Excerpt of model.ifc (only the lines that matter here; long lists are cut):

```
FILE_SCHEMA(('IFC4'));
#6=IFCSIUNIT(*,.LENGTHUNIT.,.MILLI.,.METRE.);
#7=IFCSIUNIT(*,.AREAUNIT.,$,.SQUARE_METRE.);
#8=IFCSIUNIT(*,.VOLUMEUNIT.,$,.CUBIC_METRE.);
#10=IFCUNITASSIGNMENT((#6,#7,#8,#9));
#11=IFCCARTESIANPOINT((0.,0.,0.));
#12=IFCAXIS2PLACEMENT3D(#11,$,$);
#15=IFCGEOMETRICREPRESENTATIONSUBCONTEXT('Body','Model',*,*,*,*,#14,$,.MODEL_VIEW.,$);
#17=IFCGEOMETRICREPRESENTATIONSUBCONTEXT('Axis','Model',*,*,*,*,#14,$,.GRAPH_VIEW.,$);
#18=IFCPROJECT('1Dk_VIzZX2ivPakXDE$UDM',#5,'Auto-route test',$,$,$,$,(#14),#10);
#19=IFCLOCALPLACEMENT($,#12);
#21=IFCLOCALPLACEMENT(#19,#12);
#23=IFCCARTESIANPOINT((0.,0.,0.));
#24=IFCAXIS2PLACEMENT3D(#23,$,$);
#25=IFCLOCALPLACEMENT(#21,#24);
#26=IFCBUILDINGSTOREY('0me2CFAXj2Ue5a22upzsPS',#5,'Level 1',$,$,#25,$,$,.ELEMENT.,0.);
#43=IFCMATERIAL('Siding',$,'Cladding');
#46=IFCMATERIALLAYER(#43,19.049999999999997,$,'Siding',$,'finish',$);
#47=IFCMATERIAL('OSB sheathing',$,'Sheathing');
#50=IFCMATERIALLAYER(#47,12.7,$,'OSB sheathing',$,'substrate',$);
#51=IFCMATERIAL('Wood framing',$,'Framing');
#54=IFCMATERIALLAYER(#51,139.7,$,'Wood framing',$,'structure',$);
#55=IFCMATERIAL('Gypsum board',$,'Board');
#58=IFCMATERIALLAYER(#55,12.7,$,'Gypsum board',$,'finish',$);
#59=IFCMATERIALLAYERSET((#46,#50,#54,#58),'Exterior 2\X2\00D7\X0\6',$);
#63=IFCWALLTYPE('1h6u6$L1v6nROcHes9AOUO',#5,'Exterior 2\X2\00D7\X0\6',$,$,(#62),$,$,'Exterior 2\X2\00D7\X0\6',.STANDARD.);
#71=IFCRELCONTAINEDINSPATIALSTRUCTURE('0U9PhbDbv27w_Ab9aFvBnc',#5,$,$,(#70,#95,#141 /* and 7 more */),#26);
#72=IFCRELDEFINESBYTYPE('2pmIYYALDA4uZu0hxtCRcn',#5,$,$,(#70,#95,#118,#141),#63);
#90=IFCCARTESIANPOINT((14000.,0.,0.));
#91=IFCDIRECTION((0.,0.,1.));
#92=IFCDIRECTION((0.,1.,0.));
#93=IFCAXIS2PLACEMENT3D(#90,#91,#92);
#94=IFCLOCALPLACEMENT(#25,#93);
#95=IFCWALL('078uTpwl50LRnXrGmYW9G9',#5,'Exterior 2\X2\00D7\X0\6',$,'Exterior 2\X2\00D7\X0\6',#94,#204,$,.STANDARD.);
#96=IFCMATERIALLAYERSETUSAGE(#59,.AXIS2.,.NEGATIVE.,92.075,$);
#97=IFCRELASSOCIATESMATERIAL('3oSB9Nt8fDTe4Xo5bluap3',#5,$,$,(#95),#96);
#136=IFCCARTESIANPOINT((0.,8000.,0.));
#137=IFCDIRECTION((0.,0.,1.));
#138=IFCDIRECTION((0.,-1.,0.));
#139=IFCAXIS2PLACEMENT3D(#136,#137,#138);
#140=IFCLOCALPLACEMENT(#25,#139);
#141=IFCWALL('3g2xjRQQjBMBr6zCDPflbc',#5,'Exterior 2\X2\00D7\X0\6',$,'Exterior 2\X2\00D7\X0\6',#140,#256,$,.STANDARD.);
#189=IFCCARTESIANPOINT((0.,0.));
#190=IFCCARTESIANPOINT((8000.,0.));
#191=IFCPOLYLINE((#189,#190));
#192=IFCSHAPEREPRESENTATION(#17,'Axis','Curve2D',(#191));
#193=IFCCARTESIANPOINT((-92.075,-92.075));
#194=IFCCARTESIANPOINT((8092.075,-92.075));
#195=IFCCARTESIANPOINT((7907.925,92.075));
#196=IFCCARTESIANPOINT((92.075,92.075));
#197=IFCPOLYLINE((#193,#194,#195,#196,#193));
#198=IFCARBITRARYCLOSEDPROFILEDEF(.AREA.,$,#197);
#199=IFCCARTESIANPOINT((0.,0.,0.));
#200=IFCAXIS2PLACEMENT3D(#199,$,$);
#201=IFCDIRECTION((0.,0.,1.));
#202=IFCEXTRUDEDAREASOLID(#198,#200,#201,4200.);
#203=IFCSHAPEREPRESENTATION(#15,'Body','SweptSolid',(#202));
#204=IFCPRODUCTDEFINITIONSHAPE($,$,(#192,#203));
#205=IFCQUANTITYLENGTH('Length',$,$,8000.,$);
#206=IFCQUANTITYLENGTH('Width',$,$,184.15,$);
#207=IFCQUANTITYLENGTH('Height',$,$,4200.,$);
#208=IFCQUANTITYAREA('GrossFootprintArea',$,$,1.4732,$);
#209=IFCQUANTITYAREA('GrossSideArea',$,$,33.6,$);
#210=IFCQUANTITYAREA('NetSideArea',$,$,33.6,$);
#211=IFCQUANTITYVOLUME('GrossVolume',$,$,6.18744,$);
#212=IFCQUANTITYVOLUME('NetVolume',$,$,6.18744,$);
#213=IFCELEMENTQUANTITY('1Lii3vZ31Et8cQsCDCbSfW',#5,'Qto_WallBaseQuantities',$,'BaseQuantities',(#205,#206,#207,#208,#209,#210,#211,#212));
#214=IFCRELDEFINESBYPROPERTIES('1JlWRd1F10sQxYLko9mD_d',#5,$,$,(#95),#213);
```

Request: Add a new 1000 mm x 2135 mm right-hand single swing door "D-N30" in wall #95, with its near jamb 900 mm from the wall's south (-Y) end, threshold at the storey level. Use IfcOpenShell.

```python
import numpy as np
import ifcopenshell
import ifcopenshell.api.feature
import ifcopenshell.api.geometry
import ifcopenshell.api.pset
import ifcopenshell.api.root
import ifcopenshell.api.spatial
import ifcopenshell.geom
import ifcopenshell.util.element
import ifcopenshell.util.placement
import ifcopenshell.util.representation
import ifcopenshell.util.shape
import ifcopenshell.util.unit

model = ifcopenshell.open("model.ifc")
unit_scale = ifcopenshell.util.unit.calculate_unit_scale(model)
area_scale = ifcopenshell.util.unit.calculate_unit_scale(model, "AREAUNIT")
volume_scale = ifcopenshell.util.unit.calculate_unit_scale(model, "VOLUMEUNIT")
settings = ifcopenshell.geom.settings()


def volume(element):
    """Net volume in cubic metres, openings subtracted."""
    shape = ifcopenshell.geom.create_shape(settings, element)
    return ifcopenshell.util.shape.get_volume(shape.geometry)


wall = model.by_id(95)
storey = ifcopenshell.util.element.get_container(wall, ifc_class="IfcBuildingStorey")
context = ifcopenshell.util.representation.get_context(model, "Model", "Body", "MODEL_VIEW")
before = volume(wall)

width, height, from_end, sill = 1, 2.135, 0.9, 0.0  # metres

# The wall runs along its own X axis, and the end named is its -X end.
wall_shape = ifcopenshell.geom.create_shape(settings, wall)
x, y, z = ifcopenshell.util.shape.get_vertices(wall_shape.geometry).T
start = x.min() + from_end
face, thickness = float(y.min()), float(y.max() - y.min())
wall_matrix = ifcopenshell.util.placement.get_local_placement(wall.ObjectPlacement)
level = ifcopenshell.util.placement.get_local_placement(storey.ObjectPlacement)[2, 3]


def in_wall(x, y):
    """Placement at x, y metres in the wall's axes, at sill height."""
    matrix = wall_matrix.copy()
    matrix[:, 3] = wall_matrix @ np.array([x / unit_scale, y / unit_scale, 0.0, 1.0])
    matrix[2, 3] = level + sill / unit_scale
    return matrix


# Opening: a box that overshoots both wall faces by 50 mm.
opening = ifcopenshell.api.root.create_entity(model, ifc_class="IfcOpeningElement", predefined_type="OPENING")
box = ifcopenshell.api.geometry.add_wall_representation(
    model, context=context, length=width, height=height, thickness=thickness + 0.1
)
ifcopenshell.api.geometry.assign_representation(model, product=opening, representation=box)
ifcopenshell.api.geometry.edit_object_placement(model, product=opening, matrix=in_wall(start, face - 0.05), is_si=False)
ifcopenshell.api.feature.add_feature(model, feature=opening, element=wall)

door = ifcopenshell.api.root.create_entity(model, ifc_class="IfcDoor", name="D-N30", predefined_type="DOOR")
door.OverallWidth, door.OverallHeight = width / unit_scale, height / unit_scale
door.OperationType = "SINGLE_SWING_RIGHT"
body = ifcopenshell.api.geometry.add_door_representation(
    model,
    context=context,
    overall_width=door.OverallWidth,
    overall_height=door.OverallHeight,
    operation_type="SINGLE_SWING_RIGHT",
    lining_properties={"LiningDepth": thickness / unit_scale, "ThresholdDepth": thickness / unit_scale},
)
ifcopenshell.api.geometry.assign_representation(model, product=door, representation=body)
ifcopenshell.api.spatial.assign_container(model, products=[door], relating_structure=storey)
ifcopenshell.api.feature.add_filling(model, opening=opening, element=door)

# The lining spans the wall, so the door starts at the wall face.
ifcopenshell.api.geometry.edit_object_placement(model, product=door, matrix=in_wall(start, face), is_si=False)

after = volume(wall)

# Update the wall's stored quantities.
qto = model.by_id(ifcopenshell.util.element.get_pset(wall, "Qto_WallBaseQuantities", should_inherit=False)["id"])
ifcopenshell.api.pset.edit_qto(model, qto=qto, properties={
    "NetSideArea": after / thickness / area_scale,
    "NetVolume": after / volume_scale,
})

print(f"wall volume {before:.3f} -> {after:.3f} m3")

model.write("model_rev.ifc")
```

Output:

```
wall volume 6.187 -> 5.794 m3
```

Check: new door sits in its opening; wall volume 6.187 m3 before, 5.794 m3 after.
